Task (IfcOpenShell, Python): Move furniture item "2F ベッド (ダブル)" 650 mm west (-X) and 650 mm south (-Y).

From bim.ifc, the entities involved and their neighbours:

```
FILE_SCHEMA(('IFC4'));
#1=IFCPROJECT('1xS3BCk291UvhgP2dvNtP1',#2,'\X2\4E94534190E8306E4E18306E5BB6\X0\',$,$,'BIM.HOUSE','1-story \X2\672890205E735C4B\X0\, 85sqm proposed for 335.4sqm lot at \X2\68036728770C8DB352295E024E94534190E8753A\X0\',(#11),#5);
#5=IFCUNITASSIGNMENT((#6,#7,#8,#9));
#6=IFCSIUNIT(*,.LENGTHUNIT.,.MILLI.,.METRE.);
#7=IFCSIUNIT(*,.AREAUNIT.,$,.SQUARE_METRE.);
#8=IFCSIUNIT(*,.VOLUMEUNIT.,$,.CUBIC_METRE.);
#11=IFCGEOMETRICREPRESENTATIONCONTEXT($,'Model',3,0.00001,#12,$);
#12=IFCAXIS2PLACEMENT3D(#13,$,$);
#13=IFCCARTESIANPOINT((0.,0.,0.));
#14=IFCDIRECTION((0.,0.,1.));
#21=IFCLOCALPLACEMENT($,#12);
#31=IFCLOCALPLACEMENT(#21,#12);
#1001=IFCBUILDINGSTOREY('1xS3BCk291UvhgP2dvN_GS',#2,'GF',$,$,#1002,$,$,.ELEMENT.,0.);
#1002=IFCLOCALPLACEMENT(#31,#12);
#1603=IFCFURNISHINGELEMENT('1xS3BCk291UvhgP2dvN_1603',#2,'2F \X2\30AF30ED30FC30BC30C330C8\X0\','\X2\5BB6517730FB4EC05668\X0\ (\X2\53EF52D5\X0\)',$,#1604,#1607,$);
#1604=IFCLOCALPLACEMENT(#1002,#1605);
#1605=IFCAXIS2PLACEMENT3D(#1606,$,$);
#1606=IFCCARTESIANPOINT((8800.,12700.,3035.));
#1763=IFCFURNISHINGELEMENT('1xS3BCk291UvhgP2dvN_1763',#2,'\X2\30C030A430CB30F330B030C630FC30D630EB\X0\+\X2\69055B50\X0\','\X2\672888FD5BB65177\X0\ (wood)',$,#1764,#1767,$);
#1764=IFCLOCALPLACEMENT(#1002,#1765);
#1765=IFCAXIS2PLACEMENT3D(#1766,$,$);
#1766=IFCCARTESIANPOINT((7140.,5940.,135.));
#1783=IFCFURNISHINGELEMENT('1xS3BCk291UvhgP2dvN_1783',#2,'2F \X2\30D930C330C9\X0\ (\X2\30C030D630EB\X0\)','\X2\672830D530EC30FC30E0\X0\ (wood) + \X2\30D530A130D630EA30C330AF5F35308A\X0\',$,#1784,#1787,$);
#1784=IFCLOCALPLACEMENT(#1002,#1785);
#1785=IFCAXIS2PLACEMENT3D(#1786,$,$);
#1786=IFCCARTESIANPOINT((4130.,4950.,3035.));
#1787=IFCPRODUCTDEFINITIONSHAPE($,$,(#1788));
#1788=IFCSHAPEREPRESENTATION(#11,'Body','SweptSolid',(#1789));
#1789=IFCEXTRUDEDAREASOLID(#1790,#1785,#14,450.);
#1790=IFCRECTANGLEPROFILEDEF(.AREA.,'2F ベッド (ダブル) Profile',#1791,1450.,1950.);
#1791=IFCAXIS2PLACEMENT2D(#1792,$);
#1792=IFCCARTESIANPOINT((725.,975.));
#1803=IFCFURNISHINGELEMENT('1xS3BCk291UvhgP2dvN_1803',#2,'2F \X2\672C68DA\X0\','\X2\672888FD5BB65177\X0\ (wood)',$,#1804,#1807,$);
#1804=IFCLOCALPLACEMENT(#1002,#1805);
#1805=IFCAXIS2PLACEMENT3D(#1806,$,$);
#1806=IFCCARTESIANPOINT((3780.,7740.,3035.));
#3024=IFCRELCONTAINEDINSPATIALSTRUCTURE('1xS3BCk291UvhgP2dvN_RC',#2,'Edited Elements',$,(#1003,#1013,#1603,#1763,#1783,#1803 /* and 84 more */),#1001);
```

```python
import ifcopenshell
import ifcopenshell.api.geometry
import ifcopenshell.util.placement
import ifcopenshell.util.unit

model = ifcopenshell.open("bim.ifc")
unit_scale = ifcopenshell.util.unit.calculate_unit_scale(model)

item = model.by_guid("1xS3BCk291UvhgP2dvN_1783")
matrix = ifcopenshell.util.placement.get_local_placement(item.ObjectPlacement)
matrix[0, 3] -= 0.65 / unit_scale
matrix[1, 3] -= 0.65 / unit_scale
ifcopenshell.api.geometry.edit_object_placement(model, product=item, matrix=matrix, is_si=False)

print(ifcopenshell.util.placement.get_local_placement(item.ObjectPlacement).round(3) + 0.0)

model.write("bim-out.ifc")
```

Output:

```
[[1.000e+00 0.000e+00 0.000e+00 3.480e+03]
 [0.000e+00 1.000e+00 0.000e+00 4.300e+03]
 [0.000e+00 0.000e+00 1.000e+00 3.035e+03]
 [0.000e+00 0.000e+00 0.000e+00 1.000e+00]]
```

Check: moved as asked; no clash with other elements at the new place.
